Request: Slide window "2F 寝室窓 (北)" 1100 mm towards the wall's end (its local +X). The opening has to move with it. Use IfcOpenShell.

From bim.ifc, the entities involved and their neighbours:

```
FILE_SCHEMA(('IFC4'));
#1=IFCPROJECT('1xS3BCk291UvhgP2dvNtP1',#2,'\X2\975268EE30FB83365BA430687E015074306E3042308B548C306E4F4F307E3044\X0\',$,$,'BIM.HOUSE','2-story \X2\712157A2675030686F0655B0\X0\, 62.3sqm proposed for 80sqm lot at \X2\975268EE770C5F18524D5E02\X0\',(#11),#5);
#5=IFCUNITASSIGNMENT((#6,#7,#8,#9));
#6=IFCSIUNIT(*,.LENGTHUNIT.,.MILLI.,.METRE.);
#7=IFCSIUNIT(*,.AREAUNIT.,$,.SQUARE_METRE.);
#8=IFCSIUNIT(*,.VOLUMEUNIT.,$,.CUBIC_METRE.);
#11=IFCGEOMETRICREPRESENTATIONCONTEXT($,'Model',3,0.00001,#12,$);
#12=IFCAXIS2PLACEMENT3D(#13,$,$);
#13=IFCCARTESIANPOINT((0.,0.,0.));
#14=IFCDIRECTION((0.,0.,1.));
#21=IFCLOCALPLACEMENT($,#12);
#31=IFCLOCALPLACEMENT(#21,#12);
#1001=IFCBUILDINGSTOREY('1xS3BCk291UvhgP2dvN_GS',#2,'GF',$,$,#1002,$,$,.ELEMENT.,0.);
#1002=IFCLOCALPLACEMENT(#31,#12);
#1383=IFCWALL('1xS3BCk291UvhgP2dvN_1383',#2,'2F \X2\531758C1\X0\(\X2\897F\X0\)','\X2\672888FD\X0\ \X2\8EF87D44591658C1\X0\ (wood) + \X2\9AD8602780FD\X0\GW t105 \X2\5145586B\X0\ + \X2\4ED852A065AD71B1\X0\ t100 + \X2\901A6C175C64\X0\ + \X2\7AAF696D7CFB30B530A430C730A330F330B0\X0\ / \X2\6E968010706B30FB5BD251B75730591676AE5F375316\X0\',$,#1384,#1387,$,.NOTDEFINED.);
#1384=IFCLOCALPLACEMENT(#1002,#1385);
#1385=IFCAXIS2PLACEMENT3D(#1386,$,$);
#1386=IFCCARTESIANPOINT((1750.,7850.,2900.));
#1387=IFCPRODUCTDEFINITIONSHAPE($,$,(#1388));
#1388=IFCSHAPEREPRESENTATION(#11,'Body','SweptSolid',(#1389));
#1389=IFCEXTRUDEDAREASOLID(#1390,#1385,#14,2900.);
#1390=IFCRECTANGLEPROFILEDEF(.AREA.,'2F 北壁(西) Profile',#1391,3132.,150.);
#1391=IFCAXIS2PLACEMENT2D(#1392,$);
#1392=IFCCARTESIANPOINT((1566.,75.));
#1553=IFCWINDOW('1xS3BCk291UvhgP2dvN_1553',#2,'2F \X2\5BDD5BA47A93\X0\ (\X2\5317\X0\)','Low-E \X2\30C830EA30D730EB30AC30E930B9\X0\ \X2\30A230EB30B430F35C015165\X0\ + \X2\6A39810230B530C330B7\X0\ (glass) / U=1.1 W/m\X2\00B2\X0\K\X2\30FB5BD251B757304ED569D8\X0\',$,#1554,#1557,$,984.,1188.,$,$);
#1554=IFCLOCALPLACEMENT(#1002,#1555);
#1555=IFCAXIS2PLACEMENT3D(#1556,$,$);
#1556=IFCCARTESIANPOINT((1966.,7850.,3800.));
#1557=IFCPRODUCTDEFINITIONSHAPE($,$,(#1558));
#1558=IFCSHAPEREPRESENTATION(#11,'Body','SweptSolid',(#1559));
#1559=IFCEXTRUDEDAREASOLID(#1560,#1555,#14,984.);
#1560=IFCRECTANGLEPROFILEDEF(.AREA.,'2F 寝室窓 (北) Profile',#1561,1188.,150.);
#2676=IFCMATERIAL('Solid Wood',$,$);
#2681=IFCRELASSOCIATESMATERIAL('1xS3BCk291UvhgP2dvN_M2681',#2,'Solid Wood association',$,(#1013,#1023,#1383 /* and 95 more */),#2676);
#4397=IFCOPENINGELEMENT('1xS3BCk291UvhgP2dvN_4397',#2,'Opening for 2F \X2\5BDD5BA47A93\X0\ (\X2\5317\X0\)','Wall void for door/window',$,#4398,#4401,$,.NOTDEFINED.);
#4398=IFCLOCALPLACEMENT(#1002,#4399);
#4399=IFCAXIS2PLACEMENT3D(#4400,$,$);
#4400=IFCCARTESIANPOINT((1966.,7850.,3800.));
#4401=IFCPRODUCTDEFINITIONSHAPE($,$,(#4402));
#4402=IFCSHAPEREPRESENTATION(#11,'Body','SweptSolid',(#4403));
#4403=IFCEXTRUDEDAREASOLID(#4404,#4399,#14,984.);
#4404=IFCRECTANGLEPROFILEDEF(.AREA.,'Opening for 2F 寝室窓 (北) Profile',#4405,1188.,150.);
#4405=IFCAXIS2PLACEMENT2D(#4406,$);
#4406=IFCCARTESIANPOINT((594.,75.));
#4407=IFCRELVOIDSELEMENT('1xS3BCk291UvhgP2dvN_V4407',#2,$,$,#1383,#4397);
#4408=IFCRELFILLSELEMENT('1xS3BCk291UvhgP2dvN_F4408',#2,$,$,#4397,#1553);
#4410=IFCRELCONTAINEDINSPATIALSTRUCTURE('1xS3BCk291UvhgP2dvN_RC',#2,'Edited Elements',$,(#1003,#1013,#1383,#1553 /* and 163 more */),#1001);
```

```python
import ifcopenshell
import ifcopenshell.api.geometry
import ifcopenshell.util.placement
import ifcopenshell.util.unit

model = ifcopenshell.open("bim.ifc")
unit_scale = ifcopenshell.util.unit.calculate_unit_scale(model)

window = model.by_guid("1xS3BCk291UvhgP2dvN_1553")
opening = window.FillsVoids[0].RelatingOpeningElement
wall = opening.VoidsElements[0].RelatingBuildingElement

wall_matrix = ifcopenshell.util.placement.get_local_placement(wall.ObjectPlacement)
shift = wall_matrix[:3, 0] * 1.1 / unit_scale
before = ifcopenshell.util.placement.get_local_placement(window.ObjectPlacement)[:3, 3].copy()

# The window is not placed relative to its opening, so move both.
for product in (opening, window):
    matrix = ifcopenshell.util.placement.get_local_placement(product.ObjectPlacement)
    matrix[:3, 3] += shift
    ifcopenshell.api.geometry.edit_object_placement(model, product=product, matrix=matrix, is_si=False)

after = ifcopenshell.util.placement.get_local_placement(window.ObjectPlacement)[:3, 3]
print("window moved by", (after - before).round(3) + 0.0)

model.write("bim_v2.ifc")
```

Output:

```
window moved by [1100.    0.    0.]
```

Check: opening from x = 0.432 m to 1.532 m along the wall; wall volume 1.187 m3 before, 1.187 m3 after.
